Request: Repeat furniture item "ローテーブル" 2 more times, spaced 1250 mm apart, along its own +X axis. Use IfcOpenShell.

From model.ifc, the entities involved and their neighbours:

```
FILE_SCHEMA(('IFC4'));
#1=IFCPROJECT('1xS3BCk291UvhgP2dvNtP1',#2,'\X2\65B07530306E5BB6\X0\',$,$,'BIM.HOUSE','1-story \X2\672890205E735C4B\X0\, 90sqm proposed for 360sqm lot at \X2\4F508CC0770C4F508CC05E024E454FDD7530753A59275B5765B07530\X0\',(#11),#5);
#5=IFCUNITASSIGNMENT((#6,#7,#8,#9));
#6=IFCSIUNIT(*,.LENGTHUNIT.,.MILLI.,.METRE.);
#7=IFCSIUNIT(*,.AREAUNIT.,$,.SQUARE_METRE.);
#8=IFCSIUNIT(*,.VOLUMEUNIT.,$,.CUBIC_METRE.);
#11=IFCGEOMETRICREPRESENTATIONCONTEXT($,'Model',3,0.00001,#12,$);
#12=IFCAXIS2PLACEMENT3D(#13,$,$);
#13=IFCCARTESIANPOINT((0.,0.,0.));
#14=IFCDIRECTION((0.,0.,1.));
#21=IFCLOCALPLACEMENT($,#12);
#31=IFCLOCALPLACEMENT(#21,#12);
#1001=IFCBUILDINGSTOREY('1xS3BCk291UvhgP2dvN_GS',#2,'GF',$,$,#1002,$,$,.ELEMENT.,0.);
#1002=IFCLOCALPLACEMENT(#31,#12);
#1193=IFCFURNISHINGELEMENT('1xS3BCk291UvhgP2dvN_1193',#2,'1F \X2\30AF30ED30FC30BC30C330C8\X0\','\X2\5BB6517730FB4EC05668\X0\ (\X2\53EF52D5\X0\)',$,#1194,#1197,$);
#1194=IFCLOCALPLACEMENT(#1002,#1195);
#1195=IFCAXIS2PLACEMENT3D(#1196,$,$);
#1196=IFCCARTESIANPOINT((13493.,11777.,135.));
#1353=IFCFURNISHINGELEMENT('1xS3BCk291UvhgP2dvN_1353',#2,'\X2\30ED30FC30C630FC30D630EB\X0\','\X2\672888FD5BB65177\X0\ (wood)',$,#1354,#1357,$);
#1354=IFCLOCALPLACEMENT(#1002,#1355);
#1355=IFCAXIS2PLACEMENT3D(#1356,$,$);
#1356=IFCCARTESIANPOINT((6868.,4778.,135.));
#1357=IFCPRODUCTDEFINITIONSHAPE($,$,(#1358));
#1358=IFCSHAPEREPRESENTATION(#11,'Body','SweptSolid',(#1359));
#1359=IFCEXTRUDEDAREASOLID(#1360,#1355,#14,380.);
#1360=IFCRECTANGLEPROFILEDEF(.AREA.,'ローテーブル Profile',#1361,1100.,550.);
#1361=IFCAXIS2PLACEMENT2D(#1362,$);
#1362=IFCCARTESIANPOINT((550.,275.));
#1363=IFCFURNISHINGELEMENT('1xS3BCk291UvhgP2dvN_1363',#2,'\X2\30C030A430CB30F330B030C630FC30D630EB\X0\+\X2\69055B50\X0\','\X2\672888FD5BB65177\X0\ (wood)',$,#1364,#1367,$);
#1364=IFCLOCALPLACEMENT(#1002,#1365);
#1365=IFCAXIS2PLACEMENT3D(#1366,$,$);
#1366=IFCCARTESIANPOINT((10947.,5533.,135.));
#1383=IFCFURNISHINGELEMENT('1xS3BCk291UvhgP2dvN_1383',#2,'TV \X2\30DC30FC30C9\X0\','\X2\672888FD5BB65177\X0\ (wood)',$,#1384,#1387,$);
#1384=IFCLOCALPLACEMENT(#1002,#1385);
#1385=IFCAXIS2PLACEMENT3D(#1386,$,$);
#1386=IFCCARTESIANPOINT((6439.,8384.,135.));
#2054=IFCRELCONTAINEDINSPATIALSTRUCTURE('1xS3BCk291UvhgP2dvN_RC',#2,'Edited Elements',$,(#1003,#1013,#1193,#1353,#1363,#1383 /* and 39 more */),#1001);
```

```python
import ifcopenshell
import ifcopenshell.api.geometry
import ifcopenshell.api.root
import ifcopenshell.util.element
import ifcopenshell.util.placement
import ifcopenshell.util.unit

model = ifcopenshell.open("model.ifc")
unit_scale = ifcopenshell.util.unit.calculate_unit_scale(model)


def reuse_history(source, copy):
    """copy_class also copies each property set's owner history, people and application; keep the originals."""
    for rel in copy.IsDefinedBy:
        if rel.is_a("IfcRelDefinesByProperties") and (history := rel.RelatingPropertyDefinition.OwnerHistory):
            rel.RelatingPropertyDefinition.OwnerHistory = source.OwnerHistory
            ifcopenshell.util.element.remove_deep2(model, history)


source = model.by_guid("1xS3BCk291UvhgP2dvN_1353")
base = ifcopenshell.util.placement.get_local_placement(source.ObjectPlacement)
step = base[:3, 0] * 1.25 / unit_scale

for i in range(1, 3):
    copy = ifcopenshell.api.root.copy_class(model, product=source)
    copy.Representation = ifcopenshell.util.element.copy_deep(
        model, source.Representation, exclude=["IfcGeometricRepresentationContext", "IfcRepresentationMap"]
    )
    reuse_history(source, copy)
    matrix = base.copy()
    matrix[:3, 3] += i * step
    print("added at", matrix[:3, 3].round(3) + 0.0)
    ifcopenshell.api.geometry.edit_object_placement(model, product=copy, matrix=matrix, is_si=False)

model.write("model-out.ifc")
```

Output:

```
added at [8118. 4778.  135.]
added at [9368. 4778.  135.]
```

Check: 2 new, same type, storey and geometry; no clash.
